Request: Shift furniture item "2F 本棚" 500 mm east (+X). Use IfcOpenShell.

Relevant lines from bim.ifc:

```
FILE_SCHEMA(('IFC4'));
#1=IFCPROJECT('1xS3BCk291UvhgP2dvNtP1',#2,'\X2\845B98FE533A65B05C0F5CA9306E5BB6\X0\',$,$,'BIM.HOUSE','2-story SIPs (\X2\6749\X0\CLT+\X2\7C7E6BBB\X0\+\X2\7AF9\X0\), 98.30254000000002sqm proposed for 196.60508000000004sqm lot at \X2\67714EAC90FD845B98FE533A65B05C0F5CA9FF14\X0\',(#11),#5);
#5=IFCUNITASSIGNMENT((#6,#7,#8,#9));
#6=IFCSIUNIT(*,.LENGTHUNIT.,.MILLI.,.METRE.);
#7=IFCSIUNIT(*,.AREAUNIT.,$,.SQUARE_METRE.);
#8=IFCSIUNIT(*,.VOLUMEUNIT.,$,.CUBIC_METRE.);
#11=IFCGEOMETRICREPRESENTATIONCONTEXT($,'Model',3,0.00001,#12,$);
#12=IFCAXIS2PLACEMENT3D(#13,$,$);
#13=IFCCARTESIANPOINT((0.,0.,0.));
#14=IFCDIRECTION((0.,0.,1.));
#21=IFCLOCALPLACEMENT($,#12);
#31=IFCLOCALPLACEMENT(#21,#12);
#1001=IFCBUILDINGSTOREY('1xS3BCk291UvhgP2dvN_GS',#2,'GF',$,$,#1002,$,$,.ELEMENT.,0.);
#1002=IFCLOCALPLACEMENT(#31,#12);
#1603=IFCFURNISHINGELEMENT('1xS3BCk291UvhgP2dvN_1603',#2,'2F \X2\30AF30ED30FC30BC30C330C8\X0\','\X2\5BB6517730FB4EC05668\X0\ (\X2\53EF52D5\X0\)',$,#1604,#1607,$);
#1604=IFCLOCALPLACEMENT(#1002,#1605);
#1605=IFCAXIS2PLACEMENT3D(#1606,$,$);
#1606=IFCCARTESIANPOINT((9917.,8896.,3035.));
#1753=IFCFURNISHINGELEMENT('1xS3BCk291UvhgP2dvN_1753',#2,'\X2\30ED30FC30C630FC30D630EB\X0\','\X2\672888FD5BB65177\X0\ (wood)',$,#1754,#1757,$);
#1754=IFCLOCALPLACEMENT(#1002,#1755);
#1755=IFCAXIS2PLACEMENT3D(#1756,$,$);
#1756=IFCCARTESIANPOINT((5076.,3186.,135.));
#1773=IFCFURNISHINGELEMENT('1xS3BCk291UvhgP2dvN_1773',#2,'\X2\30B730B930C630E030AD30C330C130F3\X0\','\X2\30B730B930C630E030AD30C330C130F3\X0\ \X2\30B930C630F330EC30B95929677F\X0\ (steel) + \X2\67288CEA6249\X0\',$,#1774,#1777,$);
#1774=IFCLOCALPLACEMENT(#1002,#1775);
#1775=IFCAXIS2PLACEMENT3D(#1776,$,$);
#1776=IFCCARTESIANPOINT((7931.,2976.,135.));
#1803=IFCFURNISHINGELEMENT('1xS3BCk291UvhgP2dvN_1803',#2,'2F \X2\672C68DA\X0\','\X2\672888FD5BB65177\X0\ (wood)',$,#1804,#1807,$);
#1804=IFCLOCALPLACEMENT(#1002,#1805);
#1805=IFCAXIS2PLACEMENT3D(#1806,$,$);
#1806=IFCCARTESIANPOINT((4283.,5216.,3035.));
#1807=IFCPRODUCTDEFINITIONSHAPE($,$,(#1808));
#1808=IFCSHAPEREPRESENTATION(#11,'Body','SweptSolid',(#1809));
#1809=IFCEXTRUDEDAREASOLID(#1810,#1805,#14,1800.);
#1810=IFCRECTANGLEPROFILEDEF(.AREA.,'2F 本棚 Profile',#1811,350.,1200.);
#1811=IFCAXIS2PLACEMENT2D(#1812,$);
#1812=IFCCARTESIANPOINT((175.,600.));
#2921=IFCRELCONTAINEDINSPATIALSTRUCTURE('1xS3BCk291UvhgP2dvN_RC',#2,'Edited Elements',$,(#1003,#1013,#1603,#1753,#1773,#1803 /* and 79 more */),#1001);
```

```python
import ifcopenshell
import ifcopenshell.api.geometry
import ifcopenshell.util.placement

model = ifcopenshell.open("bim.ifc")

item = model.by_guid("1xS3BCk291UvhgP2dvN_1803")
matrix = ifcopenshell.util.placement.get_local_placement(item.ObjectPlacement)
matrix[0, 3] += 500.0
ifcopenshell.api.geometry.edit_object_placement(model, product=item, matrix=matrix, is_si=False)

print(ifcopenshell.util.placement.get_local_placement(item.ObjectPlacement).round(3) + 0.0)

model.write("bim_v2.ifc")
```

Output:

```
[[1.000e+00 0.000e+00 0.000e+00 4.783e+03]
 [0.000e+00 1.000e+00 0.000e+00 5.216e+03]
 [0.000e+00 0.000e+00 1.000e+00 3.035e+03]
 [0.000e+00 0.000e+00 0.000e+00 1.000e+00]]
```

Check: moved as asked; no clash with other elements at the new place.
